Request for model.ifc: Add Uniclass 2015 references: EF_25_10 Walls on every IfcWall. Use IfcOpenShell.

First a look at what the model holds.

```python
import ifcopenshell

model = ifcopenshell.open("model.ifc")
print(model.schema)
print("classifications:", [c.Name for c in model.by_type("IfcClassification")])
for ifc_class in ("IfcDoor", "IfcRoof", "IfcStair", "IfcWall", "IfcWindow"):
    print(ifc_class, len(model.by_type(ifc_class)))
```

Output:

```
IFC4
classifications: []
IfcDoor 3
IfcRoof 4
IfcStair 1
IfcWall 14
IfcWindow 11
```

```python
import ifcopenshell
import ifcopenshell.api.classification

model = ifcopenshell.open("model.ifc")

system = ifcopenshell.api.classification.add_classification(model, classification="Uniclass 2015")

codes = {
    "IfcWall": ("EF_25_10", "Walls"),
}
for ifc_class, (code, name) in codes.items():
    products = model.by_type(ifc_class)
    ifcopenshell.api.classification.add_reference(
        model, products=products, classification=system, identification=code, name=name
    )
    print(code, len(products))

model.write("model-out.ifc")
```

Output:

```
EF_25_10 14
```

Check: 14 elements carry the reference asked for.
